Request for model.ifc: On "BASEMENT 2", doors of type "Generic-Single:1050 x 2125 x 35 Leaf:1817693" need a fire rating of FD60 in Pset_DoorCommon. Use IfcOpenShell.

First a look at what the model holds.

```python
import ifcopenshell
import ifcopenshell.util.element

model = ifcopenshell.open("model.ifc")
print(model.schema)
storey = next(s for s in model.by_type("IfcBuildingStorey") if s.Name == "BASEMENT 2")
doors = [e for e in ifcopenshell.util.element.get_decomposition(storey) if e.is_a("IfcDoor")]
seen = {}
for e in doors:
    element_type = ifcopenshell.util.element.get_type(e)
    key = (element_type.Name if element_type != e and element_type else None, ifcopenshell.util.element.get_pset(e, "Pset_DoorCommon", "FireRating"))
    seen[key] = seen.get(key, 0) + 1
for (name, value), count in sorted(seen.items(), key=str):
    print(count, "x", name, "|", value)
```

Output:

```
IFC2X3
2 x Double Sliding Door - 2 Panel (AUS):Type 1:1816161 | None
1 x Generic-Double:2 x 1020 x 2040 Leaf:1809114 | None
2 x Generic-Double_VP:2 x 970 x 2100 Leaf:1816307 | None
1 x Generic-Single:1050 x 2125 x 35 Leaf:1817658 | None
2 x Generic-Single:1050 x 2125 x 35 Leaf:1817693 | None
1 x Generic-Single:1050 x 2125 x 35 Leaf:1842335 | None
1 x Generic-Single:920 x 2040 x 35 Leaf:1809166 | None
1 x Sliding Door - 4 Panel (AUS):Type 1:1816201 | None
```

```python
import ifcopenshell
import ifcopenshell.api.pset
import ifcopenshell.util.element

model = ifcopenshell.open("model.ifc")

storey = next(s for s in model.by_type("IfcBuildingStorey") if s.Name == "BASEMENT 2")
doors = [e for e in ifcopenshell.util.element.get_decomposition(storey) if e.is_a("IfcDoor")]

count = 0
for e in doors:
    element_type = ifcopenshell.util.element.get_type(e)
    if element_type in (None, e) or element_type.Name != "Generic-Single:1050 x 2125 x 35 Leaf:1817693":
        continue
    # add_pset returns the element's existing set when there is one.
    pset = ifcopenshell.api.pset.add_pset(model, product=e, name="Pset_DoorCommon")
    ifcopenshell.api.pset.edit_pset(model, pset=pset, properties={"FireRating": "FD60"})
    count += 1

print(count, "doors updated")

model.write("model_updated.ifc")
```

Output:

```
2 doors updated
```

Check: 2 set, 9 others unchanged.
